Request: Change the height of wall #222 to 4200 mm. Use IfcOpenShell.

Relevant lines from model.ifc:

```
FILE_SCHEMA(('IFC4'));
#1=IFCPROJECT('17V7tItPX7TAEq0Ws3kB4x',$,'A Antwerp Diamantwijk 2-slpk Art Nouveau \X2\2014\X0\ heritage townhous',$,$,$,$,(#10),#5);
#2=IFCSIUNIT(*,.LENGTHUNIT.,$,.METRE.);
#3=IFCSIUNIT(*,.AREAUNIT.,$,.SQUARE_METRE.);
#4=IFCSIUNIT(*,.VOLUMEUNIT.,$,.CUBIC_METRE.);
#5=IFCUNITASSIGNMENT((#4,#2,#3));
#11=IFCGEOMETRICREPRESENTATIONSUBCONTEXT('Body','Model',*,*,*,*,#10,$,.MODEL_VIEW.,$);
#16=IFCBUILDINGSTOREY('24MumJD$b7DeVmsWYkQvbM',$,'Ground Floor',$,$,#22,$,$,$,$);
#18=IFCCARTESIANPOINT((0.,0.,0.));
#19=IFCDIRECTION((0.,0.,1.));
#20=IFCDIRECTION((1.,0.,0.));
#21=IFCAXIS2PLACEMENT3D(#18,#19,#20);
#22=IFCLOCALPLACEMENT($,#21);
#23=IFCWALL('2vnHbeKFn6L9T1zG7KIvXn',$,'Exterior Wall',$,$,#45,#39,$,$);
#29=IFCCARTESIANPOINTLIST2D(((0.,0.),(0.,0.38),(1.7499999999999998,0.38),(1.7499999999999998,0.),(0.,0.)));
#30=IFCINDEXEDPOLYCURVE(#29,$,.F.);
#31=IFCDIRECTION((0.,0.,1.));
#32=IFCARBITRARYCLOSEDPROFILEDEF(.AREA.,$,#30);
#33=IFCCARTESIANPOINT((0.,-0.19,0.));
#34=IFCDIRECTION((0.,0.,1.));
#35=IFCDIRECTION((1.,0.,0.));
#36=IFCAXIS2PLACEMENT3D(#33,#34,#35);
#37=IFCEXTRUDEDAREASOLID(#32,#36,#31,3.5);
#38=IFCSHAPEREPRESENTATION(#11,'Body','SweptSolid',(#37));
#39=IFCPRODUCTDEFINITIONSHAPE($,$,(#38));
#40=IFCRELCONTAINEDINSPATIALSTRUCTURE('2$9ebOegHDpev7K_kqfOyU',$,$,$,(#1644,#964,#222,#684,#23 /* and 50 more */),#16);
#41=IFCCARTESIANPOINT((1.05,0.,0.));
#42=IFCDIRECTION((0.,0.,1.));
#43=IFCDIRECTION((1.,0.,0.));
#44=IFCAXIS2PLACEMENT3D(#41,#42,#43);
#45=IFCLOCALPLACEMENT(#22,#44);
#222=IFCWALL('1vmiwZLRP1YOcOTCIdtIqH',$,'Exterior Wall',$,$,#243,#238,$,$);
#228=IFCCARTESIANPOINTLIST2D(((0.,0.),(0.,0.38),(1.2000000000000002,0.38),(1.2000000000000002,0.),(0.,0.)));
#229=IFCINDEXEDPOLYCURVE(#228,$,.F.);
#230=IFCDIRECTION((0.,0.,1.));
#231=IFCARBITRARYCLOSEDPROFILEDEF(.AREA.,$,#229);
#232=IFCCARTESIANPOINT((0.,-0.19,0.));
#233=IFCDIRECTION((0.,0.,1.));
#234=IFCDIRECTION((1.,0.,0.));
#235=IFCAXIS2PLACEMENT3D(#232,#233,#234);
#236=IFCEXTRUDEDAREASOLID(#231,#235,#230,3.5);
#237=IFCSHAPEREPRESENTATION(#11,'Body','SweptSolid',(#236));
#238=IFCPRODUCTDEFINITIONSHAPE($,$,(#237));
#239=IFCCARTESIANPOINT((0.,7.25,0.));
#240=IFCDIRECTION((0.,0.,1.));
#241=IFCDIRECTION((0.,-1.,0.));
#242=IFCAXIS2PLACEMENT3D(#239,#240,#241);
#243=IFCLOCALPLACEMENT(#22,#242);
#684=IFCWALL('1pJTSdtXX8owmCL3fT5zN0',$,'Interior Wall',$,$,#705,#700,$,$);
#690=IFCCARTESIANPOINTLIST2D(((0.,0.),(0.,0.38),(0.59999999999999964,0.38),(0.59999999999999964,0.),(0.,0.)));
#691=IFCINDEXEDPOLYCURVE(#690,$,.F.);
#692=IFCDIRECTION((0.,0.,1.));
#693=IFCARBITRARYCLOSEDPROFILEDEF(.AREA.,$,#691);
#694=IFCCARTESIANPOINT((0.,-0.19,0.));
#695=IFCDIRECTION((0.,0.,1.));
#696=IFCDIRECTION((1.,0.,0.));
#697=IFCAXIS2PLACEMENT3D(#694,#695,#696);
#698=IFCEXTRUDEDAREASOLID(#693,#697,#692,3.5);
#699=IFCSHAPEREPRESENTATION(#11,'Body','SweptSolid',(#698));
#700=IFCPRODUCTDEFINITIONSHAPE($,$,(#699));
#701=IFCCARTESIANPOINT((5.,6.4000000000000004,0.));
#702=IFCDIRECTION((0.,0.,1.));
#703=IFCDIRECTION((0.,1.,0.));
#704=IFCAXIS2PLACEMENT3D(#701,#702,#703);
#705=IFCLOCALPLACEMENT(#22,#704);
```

```python
import ifcopenshell
import ifcopenshell.geom
import ifcopenshell.util.representation
import ifcopenshell.util.shape

model = ifcopenshell.open("model.ifc")
settings = ifcopenshell.geom.settings()


def volume(element):
    """Net volume in cubic metres, openings subtracted."""
    shape = ifcopenshell.geom.create_shape(settings, element)
    return ifcopenshell.util.shape.get_volume(shape.geometry)


wall = model.by_guid("1vmiwZLRP1YOcOTCIdtIqH")
before = volume(wall)

body = ifcopenshell.util.representation.get_representation(wall, "Model", "Body")
solid = body.Items[0]
old_height = solid.Depth
solid.Depth = 4.2
after = volume(wall)

print(f"height {old_height:g} -> {solid.Depth:g}, volume {before:.3f} -> {after:.3f} m3")

model.write("model-out.ifc")
```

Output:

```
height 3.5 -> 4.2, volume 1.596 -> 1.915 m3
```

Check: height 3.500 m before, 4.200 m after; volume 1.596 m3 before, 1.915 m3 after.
